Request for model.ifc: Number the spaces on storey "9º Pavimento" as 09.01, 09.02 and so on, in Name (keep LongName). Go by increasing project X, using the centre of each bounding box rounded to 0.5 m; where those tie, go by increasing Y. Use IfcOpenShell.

First a look at what the model holds.

```python
import ifcopenshell
import ifcopenshell.util.element
import ifcopenshell.util.placement

model = ifcopenshell.open("model.ifc")
print(model.schema)
storey = next(s for s in model.by_type("IfcBuildingStorey") if s.Name == "9º Pavimento")
spaces = [e for e in ifcopenshell.util.element.get_decomposition(storey) if e.is_a("IfcSpace")]
for e in sorted(spaces, key=lambda e: e.id()):
    origin = ifcopenshell.util.placement.get_local_placement(e.ObjectPlacement)[:3, 3]
    print(e.id(), e.Name, e.LongName, origin.round(2) + 0.0, sep=" | ")
```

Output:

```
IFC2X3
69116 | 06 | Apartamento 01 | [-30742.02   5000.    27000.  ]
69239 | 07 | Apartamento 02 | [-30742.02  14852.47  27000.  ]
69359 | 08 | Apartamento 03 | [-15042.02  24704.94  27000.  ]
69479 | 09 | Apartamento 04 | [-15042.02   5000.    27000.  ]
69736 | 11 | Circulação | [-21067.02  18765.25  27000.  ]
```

```python
import ifcopenshell
import ifcopenshell.geom
import ifcopenshell.util.element
import ifcopenshell.util.shape

model = ifcopenshell.open("model.ifc")
settings = ifcopenshell.geom.settings()
settings.set("use-world-coords", True)


def centre(element):
    shape = ifcopenshell.geom.create_shape(settings, element)
    return ifcopenshell.util.shape.get_bbox_centroid(shape.geometry)


storey = next(s for s in model.by_type("IfcBuildingStorey") if s.Name == "9º Pavimento")
spaces = [e for e in ifcopenshell.util.element.get_decomposition(storey) if e.is_a("IfcSpace")]

# Insertion points can sit at a corner or the storey origin, so sort by the geometry (in metres).
centres = {e: centre(e) for e in spaces}
spaces.sort(key=lambda e: (round(centres[e][0] / 0.5), centres[e][1]))

for i, e in enumerate(spaces, start=1):
    number = f"09.{i:02d}"
    e.Name = number
    print(e.id(), number)

model.write("model-out.ifc")
```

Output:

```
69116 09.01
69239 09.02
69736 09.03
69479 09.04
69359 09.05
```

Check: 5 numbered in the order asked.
